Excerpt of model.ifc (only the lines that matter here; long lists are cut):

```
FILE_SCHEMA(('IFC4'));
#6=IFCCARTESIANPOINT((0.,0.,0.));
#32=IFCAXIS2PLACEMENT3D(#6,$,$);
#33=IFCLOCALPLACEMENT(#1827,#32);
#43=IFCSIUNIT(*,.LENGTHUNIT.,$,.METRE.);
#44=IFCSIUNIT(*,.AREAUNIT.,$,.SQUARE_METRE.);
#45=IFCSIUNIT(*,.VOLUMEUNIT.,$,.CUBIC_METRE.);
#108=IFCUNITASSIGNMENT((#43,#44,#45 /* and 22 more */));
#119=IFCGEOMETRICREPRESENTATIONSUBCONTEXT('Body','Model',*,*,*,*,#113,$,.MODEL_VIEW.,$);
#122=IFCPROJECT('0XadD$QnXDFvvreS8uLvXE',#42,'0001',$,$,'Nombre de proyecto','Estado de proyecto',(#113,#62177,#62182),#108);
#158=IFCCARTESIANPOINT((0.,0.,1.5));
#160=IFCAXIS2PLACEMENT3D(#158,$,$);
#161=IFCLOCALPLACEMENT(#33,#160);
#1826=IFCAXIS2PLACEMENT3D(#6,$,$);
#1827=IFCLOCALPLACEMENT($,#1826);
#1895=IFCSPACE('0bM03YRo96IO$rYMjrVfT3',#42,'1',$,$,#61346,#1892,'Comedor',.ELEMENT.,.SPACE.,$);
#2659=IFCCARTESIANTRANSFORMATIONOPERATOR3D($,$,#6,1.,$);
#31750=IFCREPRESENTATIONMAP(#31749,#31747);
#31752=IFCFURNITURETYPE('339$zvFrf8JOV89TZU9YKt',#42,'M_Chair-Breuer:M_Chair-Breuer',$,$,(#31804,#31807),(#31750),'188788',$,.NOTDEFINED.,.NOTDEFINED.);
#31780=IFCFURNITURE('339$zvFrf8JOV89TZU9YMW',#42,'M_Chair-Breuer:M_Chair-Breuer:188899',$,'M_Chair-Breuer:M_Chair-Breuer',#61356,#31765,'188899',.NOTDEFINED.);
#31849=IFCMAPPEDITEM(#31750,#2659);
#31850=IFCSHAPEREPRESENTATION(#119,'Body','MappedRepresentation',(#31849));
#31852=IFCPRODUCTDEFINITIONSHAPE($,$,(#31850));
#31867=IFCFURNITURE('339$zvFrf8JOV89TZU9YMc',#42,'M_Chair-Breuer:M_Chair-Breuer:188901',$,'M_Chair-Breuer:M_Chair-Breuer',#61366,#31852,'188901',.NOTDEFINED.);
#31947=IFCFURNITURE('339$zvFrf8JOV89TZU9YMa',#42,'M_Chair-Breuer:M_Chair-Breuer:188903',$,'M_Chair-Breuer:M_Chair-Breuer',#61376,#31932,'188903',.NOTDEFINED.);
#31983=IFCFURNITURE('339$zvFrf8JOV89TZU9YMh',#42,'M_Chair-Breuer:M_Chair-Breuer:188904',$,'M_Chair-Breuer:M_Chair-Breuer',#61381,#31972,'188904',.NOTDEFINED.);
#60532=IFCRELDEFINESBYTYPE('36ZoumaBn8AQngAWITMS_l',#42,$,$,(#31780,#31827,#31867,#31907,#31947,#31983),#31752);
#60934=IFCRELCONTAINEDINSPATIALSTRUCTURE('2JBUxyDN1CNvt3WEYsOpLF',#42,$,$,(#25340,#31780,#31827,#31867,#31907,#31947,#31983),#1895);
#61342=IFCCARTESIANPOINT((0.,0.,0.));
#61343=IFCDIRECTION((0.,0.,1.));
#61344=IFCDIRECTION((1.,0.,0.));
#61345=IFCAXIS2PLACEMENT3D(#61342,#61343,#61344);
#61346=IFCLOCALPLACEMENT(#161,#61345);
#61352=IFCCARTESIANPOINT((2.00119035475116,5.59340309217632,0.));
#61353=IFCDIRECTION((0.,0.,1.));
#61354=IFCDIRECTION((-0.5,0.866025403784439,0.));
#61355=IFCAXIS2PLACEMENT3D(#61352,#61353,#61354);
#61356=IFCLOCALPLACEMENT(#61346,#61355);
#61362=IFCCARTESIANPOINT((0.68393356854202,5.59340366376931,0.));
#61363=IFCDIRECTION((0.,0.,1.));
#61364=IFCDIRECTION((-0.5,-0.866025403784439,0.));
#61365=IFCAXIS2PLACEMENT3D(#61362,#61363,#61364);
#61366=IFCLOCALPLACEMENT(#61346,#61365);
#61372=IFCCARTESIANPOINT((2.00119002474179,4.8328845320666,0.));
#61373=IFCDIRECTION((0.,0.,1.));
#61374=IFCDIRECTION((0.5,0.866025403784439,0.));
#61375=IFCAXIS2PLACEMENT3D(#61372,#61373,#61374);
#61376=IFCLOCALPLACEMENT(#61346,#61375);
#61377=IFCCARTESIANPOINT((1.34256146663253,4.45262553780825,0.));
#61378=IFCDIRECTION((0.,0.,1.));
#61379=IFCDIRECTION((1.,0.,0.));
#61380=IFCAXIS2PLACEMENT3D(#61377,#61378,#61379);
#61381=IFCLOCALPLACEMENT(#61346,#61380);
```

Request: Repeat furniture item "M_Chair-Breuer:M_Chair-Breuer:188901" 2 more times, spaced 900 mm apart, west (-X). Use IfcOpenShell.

```python
import numpy as np
import ifcopenshell
import ifcopenshell.api.geometry
import ifcopenshell.api.root
import ifcopenshell.util.element
import ifcopenshell.util.placement
import ifcopenshell.util.unit

model = ifcopenshell.open("model.ifc")
unit_scale = ifcopenshell.util.unit.calculate_unit_scale(model)


def reuse_history(source, copy):
    """copy_class also copies each property set's owner history, people and application; keep the originals."""
    for rel in copy.IsDefinedBy:
        if rel.is_a("IfcRelDefinesByProperties") and (history := rel.RelatingPropertyDefinition.OwnerHistory):
            rel.RelatingPropertyDefinition.OwnerHistory = source.OwnerHistory
            ifcopenshell.util.element.remove_deep2(model, history)


source = model.by_id(31867)
base = ifcopenshell.util.placement.get_local_placement(source.ObjectPlacement)
step = np.array([-1.0, 0.0, 0.0]) * 0.9 / unit_scale

for i in range(1, 3):
    copy = ifcopenshell.api.root.copy_class(model, product=source)
    copy.Representation = ifcopenshell.util.element.copy_deep(
        model, source.Representation, exclude=["IfcGeometricRepresentationContext", "IfcRepresentationMap"]
    )
    copy.Name = "M_Chair-Breuer:M_Chair-Breuer"
    copy.Tag = None
    reuse_history(source, copy)
    matrix = base.copy()
    matrix[:3, 3] += i * step
    print("added at", matrix[:3, 3].round(3) + 0.0)
    ifcopenshell.api.geometry.edit_object_placement(model, product=copy, matrix=matrix, is_si=False)

model.write("model_rev.ifc")
```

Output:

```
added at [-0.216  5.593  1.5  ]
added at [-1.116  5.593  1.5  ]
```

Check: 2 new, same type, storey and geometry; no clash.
